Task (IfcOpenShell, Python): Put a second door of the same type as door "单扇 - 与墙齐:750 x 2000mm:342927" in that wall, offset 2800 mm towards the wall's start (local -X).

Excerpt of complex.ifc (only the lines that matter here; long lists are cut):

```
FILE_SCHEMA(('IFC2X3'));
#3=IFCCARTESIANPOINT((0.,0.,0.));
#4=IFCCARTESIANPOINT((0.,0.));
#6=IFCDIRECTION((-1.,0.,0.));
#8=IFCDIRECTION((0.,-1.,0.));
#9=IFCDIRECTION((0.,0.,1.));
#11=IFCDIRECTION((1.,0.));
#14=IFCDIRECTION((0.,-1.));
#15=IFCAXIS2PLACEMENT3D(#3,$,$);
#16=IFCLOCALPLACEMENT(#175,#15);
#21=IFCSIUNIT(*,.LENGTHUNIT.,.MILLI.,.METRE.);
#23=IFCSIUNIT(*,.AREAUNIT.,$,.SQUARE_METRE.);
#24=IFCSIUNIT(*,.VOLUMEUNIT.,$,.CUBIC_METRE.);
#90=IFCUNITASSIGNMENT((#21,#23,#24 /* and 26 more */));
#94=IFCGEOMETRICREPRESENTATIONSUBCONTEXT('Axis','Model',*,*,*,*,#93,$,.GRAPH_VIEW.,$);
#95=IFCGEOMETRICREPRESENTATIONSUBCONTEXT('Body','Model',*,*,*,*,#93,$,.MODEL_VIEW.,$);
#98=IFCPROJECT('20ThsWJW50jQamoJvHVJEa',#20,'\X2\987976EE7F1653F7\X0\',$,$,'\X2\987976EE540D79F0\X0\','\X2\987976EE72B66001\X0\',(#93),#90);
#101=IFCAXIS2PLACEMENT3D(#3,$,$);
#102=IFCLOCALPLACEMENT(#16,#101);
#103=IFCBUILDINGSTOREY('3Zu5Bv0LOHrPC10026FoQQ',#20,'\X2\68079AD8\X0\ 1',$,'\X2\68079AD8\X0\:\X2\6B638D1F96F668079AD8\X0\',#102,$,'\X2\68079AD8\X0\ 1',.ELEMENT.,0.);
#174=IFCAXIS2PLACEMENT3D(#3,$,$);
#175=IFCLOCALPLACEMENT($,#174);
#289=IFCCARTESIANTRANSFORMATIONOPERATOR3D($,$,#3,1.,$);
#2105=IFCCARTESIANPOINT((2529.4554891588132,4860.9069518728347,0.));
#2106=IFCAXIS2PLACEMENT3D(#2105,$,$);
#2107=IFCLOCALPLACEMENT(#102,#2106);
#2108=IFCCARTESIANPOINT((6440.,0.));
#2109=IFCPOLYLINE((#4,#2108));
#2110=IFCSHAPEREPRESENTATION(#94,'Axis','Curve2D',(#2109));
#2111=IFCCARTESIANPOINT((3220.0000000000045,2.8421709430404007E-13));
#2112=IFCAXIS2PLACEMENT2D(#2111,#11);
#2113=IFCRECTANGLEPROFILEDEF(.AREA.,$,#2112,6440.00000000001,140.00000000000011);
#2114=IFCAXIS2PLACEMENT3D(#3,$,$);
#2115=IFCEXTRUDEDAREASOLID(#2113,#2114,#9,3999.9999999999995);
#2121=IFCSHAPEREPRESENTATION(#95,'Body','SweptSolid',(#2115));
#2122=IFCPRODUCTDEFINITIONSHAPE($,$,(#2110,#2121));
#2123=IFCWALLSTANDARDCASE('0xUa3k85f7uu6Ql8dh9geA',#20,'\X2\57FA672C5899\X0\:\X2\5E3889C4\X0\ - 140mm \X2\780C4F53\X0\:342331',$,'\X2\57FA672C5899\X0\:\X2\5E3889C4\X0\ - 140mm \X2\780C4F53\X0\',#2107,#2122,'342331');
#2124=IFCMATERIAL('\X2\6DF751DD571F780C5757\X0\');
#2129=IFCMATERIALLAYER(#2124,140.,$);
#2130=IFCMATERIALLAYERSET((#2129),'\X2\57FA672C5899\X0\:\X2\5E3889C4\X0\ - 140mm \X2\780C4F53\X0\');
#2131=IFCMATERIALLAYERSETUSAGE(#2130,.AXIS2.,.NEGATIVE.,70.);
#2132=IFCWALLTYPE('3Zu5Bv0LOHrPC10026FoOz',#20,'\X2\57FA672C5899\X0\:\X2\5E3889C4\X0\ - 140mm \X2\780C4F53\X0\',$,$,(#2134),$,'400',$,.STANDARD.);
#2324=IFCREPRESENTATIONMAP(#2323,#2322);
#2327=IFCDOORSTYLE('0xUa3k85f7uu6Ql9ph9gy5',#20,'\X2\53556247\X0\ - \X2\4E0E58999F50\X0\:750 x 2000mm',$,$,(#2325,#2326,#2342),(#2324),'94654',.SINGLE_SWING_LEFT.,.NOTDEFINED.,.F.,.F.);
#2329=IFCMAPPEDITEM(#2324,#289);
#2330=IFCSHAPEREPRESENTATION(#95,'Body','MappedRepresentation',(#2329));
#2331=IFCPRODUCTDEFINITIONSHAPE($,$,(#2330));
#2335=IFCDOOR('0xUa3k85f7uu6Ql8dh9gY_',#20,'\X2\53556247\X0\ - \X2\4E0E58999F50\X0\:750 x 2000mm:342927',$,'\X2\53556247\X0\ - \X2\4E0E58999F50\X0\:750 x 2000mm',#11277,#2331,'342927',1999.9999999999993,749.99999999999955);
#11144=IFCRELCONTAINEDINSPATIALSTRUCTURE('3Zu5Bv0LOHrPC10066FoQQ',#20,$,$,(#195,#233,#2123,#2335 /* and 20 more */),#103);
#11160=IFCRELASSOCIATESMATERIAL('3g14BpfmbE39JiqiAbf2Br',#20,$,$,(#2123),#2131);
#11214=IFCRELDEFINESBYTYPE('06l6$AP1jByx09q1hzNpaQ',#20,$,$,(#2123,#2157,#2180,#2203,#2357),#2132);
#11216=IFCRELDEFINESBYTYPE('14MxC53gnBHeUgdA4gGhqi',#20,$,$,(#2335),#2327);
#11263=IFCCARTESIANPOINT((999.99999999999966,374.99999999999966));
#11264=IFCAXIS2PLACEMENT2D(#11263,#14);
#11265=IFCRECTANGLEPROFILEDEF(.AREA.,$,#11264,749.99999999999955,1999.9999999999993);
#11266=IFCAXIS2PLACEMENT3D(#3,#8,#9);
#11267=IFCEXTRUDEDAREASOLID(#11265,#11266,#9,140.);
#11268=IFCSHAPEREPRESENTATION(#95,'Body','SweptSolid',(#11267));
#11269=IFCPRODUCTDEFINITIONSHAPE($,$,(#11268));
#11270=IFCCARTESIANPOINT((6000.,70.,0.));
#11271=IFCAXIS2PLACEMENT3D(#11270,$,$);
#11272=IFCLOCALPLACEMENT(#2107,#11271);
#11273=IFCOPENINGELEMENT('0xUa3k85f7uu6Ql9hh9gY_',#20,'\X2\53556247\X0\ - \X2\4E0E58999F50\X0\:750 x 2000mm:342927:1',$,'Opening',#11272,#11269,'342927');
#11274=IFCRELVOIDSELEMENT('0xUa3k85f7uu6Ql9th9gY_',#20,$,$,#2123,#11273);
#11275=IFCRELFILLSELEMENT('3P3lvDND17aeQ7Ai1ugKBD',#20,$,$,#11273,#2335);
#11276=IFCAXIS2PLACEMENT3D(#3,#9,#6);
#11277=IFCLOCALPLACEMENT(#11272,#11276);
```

```python
import ifcopenshell
import ifcopenshell.api.feature
import ifcopenshell.api.geometry
import ifcopenshell.api.root
import ifcopenshell.geom
import ifcopenshell.util.element
import ifcopenshell.util.placement
import ifcopenshell.util.shape
import ifcopenshell.util.unit

model = ifcopenshell.open("complex.ifc")
unit_scale = ifcopenshell.util.unit.calculate_unit_scale(model)
settings = ifcopenshell.geom.settings()


def volume(element):
    """Net volume in cubic metres, openings subtracted."""
    shape = ifcopenshell.geom.create_shape(settings, element)
    return ifcopenshell.util.shape.get_volume(shape.geometry)


def reuse_history(source, copy):
    """copy_class also copies each property set's owner history, people and application; keep the originals."""
    for rel in copy.IsDefinedBy:
        if rel.is_a("IfcRelDefinesByProperties") and (history := rel.RelatingPropertyDefinition.OwnerHistory):
            rel.RelatingPropertyDefinition.OwnerHistory = source.OwnerHistory
            ifcopenshell.util.element.remove_deep2(model, history)


door = model.by_guid("0xUa3k85f7uu6Ql8dh9gY_")
opening = door.FillsVoids[0].RelatingOpeningElement
wall = opening.VoidsElements[0].RelatingBuildingElement
before = volume(wall)
shift = ifcopenshell.util.placement.get_local_placement(wall.ObjectPlacement)[:3, 0] * -2.8 / unit_scale

# copy_class copies the void relationship, type, container and properties, but no geometry.
new_opening = ifcopenshell.api.root.copy_class(model, product=opening)
new_opening.Representation = ifcopenshell.util.element.copy_deep(
    model, opening.Representation, exclude=["IfcGeometricRepresentationContext", "IfcRepresentationMap"]
)
new_opening.Name = "单扇 - 与墙齐:750 x 2000mm"
new_opening.Tag = None
new_door = ifcopenshell.api.root.copy_class(model, product=door)
new_door.Representation = ifcopenshell.util.element.copy_deep(
    model, door.Representation, exclude=["IfcGeometricRepresentationContext", "IfcRepresentationMap"]
)
new_door.Name = "单扇 - 与墙齐:750 x 2000mm"
new_door.Tag = None
reuse_history(door, new_door)
fills = ifcopenshell.api.feature.add_filling(model, opening=new_opening, element=new_door)
fills.OwnerHistory = new_door.OwnerHistory  # required in IFC2X3

for old, new in ((opening, new_opening), (door, new_door)):
    matrix = ifcopenshell.util.placement.get_local_placement(old.ObjectPlacement)
    matrix[:3, 3] += shift
    ifcopenshell.api.geometry.edit_object_placement(model, product=new, matrix=matrix, is_si=False)

after = volume(wall)

print(f"wall volume {before:.3f} -> {after:.3f} m3")

model.write("complex_v2.ifc")
```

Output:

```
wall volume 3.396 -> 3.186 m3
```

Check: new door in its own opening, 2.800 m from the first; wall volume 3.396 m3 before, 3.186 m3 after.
